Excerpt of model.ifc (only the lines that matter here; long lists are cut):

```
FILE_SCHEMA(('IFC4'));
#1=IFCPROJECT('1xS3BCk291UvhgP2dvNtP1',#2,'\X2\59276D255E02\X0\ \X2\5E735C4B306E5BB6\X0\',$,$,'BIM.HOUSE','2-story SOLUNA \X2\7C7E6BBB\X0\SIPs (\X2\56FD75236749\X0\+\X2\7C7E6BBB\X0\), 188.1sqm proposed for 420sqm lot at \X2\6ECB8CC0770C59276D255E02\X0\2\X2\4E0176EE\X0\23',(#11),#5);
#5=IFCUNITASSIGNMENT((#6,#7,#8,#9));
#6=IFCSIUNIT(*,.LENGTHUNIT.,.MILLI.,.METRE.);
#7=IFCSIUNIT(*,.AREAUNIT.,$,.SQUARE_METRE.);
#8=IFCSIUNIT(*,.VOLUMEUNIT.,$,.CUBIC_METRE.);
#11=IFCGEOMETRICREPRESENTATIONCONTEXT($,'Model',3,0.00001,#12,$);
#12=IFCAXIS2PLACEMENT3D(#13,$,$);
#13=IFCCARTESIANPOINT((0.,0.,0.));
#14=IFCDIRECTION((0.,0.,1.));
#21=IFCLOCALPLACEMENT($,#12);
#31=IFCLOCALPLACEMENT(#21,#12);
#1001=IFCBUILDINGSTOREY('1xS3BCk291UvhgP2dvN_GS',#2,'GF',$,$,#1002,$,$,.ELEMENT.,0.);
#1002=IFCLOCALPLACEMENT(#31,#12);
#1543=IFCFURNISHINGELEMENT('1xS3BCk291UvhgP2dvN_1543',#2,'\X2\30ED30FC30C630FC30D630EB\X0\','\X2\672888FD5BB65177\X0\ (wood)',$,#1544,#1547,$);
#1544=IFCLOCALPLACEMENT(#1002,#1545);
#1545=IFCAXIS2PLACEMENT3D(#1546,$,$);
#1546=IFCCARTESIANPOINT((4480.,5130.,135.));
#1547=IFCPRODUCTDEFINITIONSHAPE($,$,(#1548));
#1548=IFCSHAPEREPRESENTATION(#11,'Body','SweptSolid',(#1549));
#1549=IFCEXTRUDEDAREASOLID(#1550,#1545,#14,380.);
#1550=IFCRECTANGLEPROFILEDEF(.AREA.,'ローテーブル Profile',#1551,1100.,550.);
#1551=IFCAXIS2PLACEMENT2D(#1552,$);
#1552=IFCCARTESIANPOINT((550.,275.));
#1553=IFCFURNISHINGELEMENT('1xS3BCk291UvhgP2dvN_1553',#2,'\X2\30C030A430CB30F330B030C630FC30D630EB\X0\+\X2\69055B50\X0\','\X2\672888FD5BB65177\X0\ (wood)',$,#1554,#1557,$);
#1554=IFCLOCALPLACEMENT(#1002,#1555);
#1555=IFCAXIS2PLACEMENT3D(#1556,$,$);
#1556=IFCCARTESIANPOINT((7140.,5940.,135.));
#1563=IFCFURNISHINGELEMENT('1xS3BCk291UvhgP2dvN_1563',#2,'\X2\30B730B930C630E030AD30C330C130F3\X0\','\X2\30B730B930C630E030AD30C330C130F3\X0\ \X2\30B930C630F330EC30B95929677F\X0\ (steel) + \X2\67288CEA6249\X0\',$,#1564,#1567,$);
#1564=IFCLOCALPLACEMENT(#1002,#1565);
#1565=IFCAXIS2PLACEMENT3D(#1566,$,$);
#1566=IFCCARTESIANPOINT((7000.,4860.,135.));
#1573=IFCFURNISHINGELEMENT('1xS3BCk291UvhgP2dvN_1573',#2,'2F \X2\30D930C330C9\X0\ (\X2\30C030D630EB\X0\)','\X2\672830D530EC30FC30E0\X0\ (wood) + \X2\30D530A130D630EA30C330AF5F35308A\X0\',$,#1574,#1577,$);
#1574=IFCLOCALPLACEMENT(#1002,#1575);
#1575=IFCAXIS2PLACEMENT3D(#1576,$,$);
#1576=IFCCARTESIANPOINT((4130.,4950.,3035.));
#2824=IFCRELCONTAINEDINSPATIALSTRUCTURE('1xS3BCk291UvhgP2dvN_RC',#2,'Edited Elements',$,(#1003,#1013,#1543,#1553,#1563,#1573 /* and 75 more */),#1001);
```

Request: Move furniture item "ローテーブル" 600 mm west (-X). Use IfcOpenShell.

```python
import ifcopenshell
import ifcopenshell.api.geometry
import ifcopenshell.util.placement
import ifcopenshell.util.unit

model = ifcopenshell.open("model.ifc")
unit_scale = ifcopenshell.util.unit.calculate_unit_scale(model)

item = model.by_guid("1xS3BCk291UvhgP2dvN_1543")
matrix = ifcopenshell.util.placement.get_local_placement(item.ObjectPlacement)
matrix[0, 3] -= 0.6 / unit_scale
ifcopenshell.api.geometry.edit_object_placement(model, product=item, matrix=matrix, is_si=False)

print(ifcopenshell.util.placement.get_local_placement(item.ObjectPlacement).round(3) + 0.0)

model.write("model_edited.ifc")
```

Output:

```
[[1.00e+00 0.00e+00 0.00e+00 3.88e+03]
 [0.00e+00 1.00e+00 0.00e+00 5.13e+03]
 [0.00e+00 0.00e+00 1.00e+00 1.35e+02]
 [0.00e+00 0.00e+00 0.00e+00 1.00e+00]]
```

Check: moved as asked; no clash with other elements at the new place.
